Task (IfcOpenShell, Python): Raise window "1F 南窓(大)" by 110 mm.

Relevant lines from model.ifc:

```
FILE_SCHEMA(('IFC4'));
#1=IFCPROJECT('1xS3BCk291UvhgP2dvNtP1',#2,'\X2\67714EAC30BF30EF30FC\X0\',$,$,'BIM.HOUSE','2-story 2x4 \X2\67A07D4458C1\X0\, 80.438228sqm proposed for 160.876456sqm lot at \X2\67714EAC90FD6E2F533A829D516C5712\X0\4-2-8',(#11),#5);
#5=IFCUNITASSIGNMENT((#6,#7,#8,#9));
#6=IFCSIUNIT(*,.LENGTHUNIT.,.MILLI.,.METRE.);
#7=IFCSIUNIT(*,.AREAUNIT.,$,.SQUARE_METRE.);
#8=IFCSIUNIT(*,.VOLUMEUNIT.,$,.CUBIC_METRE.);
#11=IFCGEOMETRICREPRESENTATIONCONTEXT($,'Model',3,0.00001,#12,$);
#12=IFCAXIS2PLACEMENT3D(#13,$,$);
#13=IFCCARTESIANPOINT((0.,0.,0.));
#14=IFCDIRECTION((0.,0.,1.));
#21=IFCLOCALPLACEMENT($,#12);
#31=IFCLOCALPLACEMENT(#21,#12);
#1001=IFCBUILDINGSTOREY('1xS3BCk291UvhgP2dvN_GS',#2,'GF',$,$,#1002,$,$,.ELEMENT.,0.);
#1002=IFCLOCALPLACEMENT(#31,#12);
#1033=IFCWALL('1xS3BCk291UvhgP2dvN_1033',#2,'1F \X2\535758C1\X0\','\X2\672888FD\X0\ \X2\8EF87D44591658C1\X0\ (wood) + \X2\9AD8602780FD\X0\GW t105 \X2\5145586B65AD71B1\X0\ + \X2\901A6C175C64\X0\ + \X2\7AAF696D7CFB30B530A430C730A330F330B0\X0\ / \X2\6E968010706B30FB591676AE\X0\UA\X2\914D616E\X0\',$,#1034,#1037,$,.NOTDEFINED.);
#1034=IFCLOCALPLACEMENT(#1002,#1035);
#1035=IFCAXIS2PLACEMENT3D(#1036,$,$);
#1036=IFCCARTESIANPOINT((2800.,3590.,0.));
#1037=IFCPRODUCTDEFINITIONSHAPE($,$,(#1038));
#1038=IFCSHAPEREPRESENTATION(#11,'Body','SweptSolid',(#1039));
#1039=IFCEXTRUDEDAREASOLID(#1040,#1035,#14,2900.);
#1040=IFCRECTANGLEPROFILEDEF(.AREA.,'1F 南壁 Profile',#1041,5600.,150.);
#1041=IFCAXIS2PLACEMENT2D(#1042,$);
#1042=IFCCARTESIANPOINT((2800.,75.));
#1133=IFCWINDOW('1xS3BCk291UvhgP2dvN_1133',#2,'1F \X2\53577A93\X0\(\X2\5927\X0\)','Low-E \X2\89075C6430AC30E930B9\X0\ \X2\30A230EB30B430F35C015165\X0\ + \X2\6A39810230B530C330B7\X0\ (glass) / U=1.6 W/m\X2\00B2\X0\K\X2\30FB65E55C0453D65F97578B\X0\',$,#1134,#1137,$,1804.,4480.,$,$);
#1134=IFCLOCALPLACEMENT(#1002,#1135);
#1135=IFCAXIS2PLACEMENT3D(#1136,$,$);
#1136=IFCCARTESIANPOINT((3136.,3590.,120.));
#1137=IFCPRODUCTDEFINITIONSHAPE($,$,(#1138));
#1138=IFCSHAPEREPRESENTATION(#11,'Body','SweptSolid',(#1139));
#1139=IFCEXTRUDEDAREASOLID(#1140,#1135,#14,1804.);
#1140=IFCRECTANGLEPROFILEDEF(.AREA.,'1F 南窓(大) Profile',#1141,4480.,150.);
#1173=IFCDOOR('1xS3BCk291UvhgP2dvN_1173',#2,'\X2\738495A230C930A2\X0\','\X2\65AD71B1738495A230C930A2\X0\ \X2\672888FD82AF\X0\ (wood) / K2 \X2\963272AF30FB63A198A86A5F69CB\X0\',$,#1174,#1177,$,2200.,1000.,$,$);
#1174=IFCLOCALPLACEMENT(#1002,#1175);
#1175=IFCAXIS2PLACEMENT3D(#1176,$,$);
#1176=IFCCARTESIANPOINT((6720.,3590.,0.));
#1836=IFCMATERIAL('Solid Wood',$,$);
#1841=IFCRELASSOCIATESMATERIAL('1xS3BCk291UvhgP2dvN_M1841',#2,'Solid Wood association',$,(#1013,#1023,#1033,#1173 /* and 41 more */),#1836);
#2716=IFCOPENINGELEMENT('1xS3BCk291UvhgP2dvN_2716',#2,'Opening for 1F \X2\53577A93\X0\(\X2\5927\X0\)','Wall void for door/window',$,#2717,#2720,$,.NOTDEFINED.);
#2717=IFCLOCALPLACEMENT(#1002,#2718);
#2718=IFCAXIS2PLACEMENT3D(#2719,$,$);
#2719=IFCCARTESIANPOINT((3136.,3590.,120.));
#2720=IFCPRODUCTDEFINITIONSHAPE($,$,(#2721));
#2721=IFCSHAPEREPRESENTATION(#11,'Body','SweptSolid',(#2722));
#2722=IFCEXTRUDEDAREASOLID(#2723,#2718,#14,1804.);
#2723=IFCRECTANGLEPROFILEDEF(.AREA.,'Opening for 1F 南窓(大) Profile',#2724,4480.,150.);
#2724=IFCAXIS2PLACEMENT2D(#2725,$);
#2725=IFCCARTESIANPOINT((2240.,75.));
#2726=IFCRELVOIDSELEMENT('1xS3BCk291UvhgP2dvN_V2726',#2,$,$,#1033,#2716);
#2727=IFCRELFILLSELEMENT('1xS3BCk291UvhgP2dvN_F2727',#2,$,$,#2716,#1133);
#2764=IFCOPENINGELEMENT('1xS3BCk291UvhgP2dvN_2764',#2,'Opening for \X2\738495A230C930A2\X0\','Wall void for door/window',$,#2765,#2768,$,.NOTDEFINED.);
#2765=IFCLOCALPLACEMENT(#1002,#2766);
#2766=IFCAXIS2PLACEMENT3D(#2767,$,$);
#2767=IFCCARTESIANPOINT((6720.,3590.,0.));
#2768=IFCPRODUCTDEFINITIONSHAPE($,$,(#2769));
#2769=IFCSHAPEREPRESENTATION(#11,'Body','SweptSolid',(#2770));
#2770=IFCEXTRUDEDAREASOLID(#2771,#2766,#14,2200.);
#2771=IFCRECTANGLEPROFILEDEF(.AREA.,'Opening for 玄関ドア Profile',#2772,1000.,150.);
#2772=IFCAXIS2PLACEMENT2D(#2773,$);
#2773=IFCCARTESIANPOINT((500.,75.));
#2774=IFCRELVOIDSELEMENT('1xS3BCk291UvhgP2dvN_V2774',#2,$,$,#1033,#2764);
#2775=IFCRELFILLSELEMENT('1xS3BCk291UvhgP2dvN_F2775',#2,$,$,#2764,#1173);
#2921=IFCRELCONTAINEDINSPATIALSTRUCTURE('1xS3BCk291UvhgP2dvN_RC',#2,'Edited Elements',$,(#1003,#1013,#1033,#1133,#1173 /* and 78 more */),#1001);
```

```python
import numpy as np
import ifcopenshell
import ifcopenshell.api.geometry
import ifcopenshell.util.placement
import ifcopenshell.util.unit

model = ifcopenshell.open("model.ifc")
unit_scale = ifcopenshell.util.unit.calculate_unit_scale(model)

window = model.by_guid("1xS3BCk291UvhgP2dvN_1133")
opening = window.FillsVoids[0].RelatingOpeningElement
dz = 110.0

shift = np.array([0.0, 0.0, dz])
# The window is not placed relative to its opening, so move both.
for product in (opening, window):
    matrix = ifcopenshell.util.placement.get_local_placement(product.ObjectPlacement)
    matrix[:3, 3] += shift
    ifcopenshell.api.geometry.edit_object_placement(model, product=product, matrix=matrix, is_si=False)

print(f"moved by {dz * unit_scale:+.3f} m")

model.write("model_edited.ifc")
```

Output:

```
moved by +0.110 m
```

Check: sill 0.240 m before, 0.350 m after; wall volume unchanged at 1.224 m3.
